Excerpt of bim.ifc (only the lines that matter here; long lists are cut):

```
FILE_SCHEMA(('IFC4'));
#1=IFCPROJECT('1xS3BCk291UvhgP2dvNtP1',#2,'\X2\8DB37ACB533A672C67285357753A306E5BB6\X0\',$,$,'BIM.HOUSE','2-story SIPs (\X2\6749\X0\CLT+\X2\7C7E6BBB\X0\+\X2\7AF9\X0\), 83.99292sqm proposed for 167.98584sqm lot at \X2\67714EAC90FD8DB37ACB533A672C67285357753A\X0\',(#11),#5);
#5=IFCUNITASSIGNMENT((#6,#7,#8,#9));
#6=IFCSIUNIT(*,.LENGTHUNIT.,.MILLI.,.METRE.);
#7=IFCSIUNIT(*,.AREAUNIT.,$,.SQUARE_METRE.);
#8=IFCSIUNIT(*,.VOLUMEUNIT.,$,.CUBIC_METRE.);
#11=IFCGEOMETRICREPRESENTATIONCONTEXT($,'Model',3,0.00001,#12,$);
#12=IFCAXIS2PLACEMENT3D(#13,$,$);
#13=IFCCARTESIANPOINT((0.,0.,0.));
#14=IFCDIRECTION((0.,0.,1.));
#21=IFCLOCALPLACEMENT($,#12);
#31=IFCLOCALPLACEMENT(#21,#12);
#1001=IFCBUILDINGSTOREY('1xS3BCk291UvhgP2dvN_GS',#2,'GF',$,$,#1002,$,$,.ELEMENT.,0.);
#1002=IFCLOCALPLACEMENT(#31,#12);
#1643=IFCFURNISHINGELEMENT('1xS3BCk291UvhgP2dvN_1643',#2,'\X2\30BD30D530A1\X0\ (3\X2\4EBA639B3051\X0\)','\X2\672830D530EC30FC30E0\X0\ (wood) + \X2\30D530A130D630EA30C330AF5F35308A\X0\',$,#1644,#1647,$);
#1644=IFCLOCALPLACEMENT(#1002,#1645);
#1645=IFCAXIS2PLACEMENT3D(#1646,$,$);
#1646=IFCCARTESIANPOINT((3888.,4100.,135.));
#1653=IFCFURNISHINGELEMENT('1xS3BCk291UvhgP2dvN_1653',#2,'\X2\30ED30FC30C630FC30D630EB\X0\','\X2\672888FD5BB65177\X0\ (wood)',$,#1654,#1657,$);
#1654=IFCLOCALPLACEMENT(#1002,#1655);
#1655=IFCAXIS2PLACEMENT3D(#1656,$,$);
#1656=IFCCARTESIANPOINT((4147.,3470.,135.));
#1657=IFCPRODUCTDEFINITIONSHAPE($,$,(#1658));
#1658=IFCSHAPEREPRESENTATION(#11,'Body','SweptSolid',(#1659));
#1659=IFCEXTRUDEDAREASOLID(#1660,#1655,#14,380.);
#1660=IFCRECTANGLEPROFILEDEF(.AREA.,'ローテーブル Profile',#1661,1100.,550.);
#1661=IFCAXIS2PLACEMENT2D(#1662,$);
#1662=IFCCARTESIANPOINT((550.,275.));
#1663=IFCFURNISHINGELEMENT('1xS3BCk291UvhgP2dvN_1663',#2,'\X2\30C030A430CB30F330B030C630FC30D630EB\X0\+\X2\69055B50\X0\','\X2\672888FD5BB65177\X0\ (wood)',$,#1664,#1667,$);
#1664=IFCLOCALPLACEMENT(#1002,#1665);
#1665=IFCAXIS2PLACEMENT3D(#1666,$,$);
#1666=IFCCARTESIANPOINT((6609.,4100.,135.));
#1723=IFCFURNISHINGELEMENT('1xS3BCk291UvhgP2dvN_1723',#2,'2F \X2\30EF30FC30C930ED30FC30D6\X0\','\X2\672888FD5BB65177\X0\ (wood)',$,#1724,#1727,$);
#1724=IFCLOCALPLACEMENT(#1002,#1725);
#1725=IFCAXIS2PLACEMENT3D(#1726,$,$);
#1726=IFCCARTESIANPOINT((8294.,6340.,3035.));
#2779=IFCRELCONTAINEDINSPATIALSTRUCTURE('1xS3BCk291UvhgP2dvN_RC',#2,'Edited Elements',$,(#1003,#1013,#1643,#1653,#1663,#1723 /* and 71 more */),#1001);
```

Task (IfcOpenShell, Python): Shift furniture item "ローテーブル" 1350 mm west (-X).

```python
import ifcopenshell
import ifcopenshell.api.geometry
import ifcopenshell.util.placement
import ifcopenshell.util.unit

model = ifcopenshell.open("bim.ifc")
unit_scale = ifcopenshell.util.unit.calculate_unit_scale(model)

item = model.by_id(1653)
matrix = ifcopenshell.util.placement.get_local_placement(item.ObjectPlacement)
matrix[0, 3] -= 1.35 / unit_scale
ifcopenshell.api.geometry.edit_object_placement(model, product=item, matrix=matrix, is_si=False)

print(ifcopenshell.util.placement.get_local_placement(item.ObjectPlacement).round(3) + 0.0)

model.write("bim_rev.ifc")
```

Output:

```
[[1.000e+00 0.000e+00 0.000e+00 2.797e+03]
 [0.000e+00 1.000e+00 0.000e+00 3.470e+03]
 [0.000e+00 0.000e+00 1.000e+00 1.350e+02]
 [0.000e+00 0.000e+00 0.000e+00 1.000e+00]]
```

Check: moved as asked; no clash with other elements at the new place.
